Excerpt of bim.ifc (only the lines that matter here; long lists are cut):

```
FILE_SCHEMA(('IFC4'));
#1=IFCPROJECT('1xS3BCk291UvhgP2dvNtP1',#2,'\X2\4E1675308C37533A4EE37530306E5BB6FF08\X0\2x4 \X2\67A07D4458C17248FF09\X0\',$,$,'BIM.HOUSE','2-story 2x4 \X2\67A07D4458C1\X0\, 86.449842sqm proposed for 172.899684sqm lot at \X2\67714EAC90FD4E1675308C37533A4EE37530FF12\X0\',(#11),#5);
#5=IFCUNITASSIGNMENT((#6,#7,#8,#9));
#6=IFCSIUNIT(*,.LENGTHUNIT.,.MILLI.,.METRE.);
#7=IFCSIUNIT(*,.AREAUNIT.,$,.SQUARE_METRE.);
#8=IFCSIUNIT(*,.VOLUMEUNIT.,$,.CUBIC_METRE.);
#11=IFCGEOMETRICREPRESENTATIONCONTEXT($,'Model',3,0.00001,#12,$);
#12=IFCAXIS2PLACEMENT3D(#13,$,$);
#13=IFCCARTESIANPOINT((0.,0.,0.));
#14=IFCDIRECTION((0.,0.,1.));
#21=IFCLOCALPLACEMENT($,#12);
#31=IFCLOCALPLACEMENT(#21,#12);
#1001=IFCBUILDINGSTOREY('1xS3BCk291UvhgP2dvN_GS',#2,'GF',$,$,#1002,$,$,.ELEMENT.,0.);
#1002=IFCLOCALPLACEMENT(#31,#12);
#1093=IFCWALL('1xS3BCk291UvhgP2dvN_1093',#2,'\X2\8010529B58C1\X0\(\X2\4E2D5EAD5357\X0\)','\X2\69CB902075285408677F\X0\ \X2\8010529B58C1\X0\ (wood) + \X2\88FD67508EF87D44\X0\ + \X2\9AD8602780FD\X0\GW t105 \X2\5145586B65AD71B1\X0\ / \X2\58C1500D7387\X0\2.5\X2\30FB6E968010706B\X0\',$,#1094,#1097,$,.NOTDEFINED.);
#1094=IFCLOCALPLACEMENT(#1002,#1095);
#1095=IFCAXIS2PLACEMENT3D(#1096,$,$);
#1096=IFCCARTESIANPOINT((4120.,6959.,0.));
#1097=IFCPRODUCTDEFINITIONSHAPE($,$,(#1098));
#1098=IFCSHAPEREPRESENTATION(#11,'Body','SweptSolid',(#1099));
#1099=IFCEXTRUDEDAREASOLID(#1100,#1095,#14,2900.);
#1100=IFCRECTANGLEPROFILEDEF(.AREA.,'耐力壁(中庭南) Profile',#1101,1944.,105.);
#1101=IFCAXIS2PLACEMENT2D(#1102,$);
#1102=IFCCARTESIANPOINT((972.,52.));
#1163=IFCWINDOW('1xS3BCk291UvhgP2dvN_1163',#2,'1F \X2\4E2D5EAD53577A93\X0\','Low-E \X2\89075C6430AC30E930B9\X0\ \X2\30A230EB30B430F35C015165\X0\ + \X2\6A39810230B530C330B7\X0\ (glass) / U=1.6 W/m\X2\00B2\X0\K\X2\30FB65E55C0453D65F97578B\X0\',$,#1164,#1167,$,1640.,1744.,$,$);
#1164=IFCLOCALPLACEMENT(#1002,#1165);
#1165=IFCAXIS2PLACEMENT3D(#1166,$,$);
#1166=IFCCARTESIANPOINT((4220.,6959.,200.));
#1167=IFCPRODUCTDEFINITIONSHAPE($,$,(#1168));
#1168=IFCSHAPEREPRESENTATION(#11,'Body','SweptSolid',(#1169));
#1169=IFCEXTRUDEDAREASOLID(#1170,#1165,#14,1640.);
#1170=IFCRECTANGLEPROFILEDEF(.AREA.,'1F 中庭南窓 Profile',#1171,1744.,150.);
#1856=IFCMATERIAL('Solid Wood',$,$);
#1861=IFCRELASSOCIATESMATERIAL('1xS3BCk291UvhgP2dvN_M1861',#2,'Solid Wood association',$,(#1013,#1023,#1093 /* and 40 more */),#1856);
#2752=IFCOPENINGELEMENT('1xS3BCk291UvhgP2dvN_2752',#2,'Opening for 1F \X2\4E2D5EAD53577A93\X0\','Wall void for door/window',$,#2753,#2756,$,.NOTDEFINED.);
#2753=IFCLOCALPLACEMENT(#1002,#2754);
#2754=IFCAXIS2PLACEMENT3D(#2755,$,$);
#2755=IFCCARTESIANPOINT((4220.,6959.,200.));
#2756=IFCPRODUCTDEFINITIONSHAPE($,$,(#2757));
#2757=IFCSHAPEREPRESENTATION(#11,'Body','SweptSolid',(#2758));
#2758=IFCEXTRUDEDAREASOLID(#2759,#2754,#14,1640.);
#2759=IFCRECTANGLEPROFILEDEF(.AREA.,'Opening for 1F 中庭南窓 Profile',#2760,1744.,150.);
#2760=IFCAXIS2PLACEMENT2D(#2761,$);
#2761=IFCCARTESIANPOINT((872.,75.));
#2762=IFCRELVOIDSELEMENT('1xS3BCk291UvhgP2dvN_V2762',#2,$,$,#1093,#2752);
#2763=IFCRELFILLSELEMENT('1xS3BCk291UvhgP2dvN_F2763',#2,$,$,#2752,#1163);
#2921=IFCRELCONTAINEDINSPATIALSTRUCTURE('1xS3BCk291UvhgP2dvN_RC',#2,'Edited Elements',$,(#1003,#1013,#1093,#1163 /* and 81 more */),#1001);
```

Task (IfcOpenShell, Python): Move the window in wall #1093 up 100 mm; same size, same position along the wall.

```python
import numpy as np
import ifcopenshell
import ifcopenshell.api.geometry
import ifcopenshell.util.placement
import ifcopenshell.util.unit

model = ifcopenshell.open("bim.ifc")
unit_scale = ifcopenshell.util.unit.calculate_unit_scale(model)

window = model.by_guid("1xS3BCk291UvhgP2dvN_1163")
opening = window.FillsVoids[0].RelatingOpeningElement
dz = 0.1 / unit_scale

shift = np.array([0.0, 0.0, dz])
# The window is not placed relative to its opening, so move both.
for product in (opening, window):
    matrix = ifcopenshell.util.placement.get_local_placement(product.ObjectPlacement)
    matrix[:3, 3] += shift
    ifcopenshell.api.geometry.edit_object_placement(model, product=product, matrix=matrix, is_si=False)

print(f"moved by {dz * unit_scale:+.3f} m")

model.write("bim_v2.ifc")
```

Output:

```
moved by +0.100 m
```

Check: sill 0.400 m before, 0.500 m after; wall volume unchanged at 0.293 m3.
